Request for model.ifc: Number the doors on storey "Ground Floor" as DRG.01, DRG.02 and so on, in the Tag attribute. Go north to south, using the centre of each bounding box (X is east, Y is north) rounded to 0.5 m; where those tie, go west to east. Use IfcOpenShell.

First a look at what the model holds.

```python
import ifcopenshell
import ifcopenshell.util.element
import ifcopenshell.util.placement

model = ifcopenshell.open("model.ifc")
print(model.schema)
storey = next(s for s in model.by_type("IfcBuildingStorey") if s.Name == "Ground Floor")
doors = [e for e in ifcopenshell.util.element.get_decomposition(storey) if e.is_a("IfcDoor")]
for e in sorted(doors, key=lambda e: e.id()):
    origin = ifcopenshell.util.placement.get_local_placement(e.ObjectPlacement)[:3, 3]
    print(e.id(), e.Tag, e.Name, origin.round(2) + 0.0, sep=" | ")
```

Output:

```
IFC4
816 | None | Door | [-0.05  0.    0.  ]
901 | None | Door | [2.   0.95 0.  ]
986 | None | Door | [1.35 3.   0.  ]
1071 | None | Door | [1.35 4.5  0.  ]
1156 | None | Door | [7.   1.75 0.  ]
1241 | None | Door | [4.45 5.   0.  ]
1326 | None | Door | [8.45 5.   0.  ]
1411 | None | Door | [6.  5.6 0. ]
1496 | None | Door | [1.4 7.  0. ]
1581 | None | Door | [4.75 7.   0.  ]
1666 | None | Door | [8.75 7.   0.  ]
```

```python
import ifcopenshell
import ifcopenshell.geom
import ifcopenshell.util.element
import ifcopenshell.util.shape

model = ifcopenshell.open("model.ifc")
settings = ifcopenshell.geom.settings()
settings.set("use-world-coords", True)


def centre(element):
    shape = ifcopenshell.geom.create_shape(settings, element)
    return ifcopenshell.util.shape.get_bbox_centroid(shape.geometry)


storey = next(s for s in model.by_type("IfcBuildingStorey") if s.Name == "Ground Floor")
doors = [e for e in ifcopenshell.util.element.get_decomposition(storey) if e.is_a("IfcDoor")]

# Insertion points can sit at a corner or the storey origin, so sort by the geometry (in metres).
centres = {e: centre(e) for e in doors}
doors.sort(key=lambda e: (-round(centres[e][1] / 0.5), centres[e][0]))

for i, e in enumerate(doors, start=1):
    number = f"DRG.{i:02d}"
    e.Tag = number
    print(e.id(), number)

model.write("model-out.ifc")
```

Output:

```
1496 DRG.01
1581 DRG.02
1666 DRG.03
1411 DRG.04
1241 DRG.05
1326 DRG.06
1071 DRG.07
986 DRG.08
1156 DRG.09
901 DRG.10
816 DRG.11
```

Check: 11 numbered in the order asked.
